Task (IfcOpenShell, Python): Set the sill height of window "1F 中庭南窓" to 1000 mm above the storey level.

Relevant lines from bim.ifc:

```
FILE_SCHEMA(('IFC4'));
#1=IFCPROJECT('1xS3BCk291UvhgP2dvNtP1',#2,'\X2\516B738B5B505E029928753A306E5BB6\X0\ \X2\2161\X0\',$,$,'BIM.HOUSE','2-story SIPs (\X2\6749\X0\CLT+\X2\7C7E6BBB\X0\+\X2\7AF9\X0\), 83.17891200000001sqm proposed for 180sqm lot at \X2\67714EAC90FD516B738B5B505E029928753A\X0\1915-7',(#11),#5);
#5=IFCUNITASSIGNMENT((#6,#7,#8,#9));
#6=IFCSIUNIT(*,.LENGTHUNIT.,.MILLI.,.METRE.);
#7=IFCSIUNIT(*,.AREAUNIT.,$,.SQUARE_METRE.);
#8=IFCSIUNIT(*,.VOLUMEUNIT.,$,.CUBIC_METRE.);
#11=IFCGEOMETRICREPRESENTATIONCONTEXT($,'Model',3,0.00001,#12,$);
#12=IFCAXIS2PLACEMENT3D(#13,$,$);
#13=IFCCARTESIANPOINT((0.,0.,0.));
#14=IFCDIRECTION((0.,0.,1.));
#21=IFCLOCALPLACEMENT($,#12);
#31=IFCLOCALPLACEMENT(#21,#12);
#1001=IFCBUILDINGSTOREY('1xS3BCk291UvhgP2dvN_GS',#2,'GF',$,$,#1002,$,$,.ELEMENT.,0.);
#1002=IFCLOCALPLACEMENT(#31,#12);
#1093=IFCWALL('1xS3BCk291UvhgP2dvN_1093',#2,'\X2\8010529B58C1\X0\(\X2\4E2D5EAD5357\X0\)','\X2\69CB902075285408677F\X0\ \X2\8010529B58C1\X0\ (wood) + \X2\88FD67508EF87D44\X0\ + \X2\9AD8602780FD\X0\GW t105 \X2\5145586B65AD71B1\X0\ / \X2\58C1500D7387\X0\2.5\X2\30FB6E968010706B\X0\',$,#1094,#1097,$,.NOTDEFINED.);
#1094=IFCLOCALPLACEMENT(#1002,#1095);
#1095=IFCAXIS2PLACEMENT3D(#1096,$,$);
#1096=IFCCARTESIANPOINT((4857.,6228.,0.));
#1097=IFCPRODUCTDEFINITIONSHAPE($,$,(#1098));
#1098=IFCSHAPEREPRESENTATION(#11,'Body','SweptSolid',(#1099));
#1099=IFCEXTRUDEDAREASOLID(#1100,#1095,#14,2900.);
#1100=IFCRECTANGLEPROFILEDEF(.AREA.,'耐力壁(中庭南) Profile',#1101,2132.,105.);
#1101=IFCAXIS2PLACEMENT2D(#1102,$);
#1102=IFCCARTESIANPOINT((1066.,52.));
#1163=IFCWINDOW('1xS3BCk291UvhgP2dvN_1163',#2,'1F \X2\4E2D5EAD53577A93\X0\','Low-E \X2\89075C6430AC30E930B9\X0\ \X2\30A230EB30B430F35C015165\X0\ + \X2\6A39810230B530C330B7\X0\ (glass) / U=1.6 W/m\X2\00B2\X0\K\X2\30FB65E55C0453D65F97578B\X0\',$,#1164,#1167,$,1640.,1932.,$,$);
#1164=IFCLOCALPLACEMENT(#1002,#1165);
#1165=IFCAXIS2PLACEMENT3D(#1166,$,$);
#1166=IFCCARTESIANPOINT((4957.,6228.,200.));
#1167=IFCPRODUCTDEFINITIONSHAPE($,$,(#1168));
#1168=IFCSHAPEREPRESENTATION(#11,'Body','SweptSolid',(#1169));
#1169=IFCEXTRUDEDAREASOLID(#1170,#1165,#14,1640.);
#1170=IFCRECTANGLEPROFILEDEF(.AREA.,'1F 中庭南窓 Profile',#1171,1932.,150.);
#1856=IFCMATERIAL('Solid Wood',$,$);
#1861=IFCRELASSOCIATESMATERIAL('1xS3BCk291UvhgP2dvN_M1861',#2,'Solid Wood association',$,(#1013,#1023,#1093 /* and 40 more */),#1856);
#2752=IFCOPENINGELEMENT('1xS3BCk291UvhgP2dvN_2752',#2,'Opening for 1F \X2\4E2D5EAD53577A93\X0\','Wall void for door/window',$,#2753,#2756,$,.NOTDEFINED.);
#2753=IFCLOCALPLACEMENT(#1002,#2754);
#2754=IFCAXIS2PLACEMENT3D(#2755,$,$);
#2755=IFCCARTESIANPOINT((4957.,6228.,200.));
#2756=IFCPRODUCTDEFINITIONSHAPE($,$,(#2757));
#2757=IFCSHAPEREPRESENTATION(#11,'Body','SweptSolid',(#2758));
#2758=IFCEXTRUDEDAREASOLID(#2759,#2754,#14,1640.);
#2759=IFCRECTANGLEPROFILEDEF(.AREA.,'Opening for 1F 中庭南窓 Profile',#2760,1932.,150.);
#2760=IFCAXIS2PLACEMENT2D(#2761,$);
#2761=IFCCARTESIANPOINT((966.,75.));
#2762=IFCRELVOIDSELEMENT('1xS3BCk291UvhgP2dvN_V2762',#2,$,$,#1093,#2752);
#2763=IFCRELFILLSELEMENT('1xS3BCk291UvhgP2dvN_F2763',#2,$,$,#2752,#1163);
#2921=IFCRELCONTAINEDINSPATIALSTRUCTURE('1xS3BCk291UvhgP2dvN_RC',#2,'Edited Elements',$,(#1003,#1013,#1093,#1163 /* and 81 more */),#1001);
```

```python
import numpy as np
import ifcopenshell
import ifcopenshell.api.geometry
import ifcopenshell.geom
import ifcopenshell.util.element
import ifcopenshell.util.placement
import ifcopenshell.util.shape
import ifcopenshell.util.unit

model = ifcopenshell.open("bim.ifc")
unit_scale = ifcopenshell.util.unit.calculate_unit_scale(model)

window = model.by_guid("1xS3BCk291UvhgP2dvN_1163")
opening = window.FillsVoids[0].RelatingOpeningElement
storey = ifcopenshell.util.element.get_container(window, ifc_class="IfcBuildingStorey")
level = ifcopenshell.util.placement.get_local_placement(storey.ObjectPlacement)[2, 3]

# The opening's origin need not be at the sill, so measure its lowest point.
shape = ifcopenshell.geom.create_shape(ifcopenshell.geom.settings(), opening)
bottom = ifcopenshell.util.shape.get_shape_bottom_elevation(shape, shape.geometry) / unit_scale
dz = level + 1000.0 - bottom

shift = np.array([0.0, 0.0, dz])
# The window is not placed relative to its opening, so move both.
for product in (opening, window):
    matrix = ifcopenshell.util.placement.get_local_placement(product.ObjectPlacement)
    matrix[:3, 3] += shift
    ifcopenshell.api.geometry.edit_object_placement(model, product=product, matrix=matrix, is_si=False)

print(f"moved by {dz * unit_scale:+.3f} m")

model.write("bim_updated.ifc")
```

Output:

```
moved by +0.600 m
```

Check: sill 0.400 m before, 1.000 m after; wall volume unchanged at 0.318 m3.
